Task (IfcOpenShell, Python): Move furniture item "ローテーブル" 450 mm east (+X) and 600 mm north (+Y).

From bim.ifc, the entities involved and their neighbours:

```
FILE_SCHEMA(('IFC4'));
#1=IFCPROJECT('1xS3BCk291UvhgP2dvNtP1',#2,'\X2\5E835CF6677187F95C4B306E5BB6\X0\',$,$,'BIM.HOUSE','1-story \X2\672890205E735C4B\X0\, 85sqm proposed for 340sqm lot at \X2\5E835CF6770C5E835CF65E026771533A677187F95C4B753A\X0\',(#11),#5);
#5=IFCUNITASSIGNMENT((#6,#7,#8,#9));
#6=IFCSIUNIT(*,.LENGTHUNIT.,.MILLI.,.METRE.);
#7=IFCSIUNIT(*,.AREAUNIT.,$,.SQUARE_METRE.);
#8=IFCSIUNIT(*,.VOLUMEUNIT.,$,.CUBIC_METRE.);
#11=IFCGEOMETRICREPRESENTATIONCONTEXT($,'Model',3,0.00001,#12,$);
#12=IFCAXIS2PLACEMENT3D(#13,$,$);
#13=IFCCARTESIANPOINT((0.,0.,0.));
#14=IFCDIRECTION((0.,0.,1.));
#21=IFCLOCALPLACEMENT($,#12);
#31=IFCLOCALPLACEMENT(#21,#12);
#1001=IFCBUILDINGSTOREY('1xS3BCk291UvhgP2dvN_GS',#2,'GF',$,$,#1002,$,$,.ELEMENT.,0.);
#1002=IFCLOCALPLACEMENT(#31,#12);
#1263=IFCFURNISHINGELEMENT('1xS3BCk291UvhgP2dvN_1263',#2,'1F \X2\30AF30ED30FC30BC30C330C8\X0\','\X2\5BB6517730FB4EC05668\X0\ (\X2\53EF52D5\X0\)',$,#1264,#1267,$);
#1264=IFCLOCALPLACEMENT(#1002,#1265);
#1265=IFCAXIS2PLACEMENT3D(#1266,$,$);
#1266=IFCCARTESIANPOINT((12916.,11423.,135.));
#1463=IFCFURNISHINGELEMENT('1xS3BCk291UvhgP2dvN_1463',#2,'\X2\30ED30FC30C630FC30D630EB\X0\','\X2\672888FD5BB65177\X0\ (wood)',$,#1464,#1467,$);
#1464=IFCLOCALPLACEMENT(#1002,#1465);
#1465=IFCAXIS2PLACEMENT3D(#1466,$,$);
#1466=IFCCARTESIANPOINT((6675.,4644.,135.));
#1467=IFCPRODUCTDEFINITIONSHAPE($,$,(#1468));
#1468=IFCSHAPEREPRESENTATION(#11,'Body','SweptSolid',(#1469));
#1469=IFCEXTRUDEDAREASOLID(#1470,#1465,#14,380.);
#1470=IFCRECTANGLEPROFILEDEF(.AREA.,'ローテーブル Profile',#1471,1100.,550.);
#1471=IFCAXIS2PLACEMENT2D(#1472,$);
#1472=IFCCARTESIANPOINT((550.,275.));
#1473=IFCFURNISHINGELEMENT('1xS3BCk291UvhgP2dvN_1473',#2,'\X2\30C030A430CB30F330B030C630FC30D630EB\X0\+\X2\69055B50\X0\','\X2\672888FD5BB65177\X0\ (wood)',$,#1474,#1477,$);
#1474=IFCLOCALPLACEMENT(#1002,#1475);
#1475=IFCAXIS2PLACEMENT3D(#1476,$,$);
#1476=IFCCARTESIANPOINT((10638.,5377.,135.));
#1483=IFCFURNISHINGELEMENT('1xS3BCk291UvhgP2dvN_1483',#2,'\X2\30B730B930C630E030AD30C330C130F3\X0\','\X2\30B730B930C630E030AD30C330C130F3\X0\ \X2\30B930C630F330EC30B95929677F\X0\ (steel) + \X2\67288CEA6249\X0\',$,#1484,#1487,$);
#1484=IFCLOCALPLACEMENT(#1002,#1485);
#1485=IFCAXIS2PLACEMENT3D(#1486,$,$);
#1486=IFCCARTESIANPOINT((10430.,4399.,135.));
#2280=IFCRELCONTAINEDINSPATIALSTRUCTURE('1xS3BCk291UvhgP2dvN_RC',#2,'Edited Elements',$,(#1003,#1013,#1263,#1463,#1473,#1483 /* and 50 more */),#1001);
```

```python
import ifcopenshell
import ifcopenshell.api.geometry
import ifcopenshell.util.placement
import ifcopenshell.util.unit

model = ifcopenshell.open("bim.ifc")
unit_scale = ifcopenshell.util.unit.calculate_unit_scale(model)

item = model.by_id(1463)
matrix = ifcopenshell.util.placement.get_local_placement(item.ObjectPlacement)
matrix[0, 3] += 0.45 / unit_scale
matrix[1, 3] += 0.6 / unit_scale
ifcopenshell.api.geometry.edit_object_placement(model, product=item, matrix=matrix, is_si=False)

print(ifcopenshell.util.placement.get_local_placement(item.ObjectPlacement).round(3) + 0.0)

model.write("bim_updated.ifc")
```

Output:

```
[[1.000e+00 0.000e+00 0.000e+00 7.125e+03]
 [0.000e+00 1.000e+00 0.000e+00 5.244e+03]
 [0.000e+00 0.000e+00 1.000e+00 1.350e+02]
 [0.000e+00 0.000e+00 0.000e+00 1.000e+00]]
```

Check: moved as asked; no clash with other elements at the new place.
